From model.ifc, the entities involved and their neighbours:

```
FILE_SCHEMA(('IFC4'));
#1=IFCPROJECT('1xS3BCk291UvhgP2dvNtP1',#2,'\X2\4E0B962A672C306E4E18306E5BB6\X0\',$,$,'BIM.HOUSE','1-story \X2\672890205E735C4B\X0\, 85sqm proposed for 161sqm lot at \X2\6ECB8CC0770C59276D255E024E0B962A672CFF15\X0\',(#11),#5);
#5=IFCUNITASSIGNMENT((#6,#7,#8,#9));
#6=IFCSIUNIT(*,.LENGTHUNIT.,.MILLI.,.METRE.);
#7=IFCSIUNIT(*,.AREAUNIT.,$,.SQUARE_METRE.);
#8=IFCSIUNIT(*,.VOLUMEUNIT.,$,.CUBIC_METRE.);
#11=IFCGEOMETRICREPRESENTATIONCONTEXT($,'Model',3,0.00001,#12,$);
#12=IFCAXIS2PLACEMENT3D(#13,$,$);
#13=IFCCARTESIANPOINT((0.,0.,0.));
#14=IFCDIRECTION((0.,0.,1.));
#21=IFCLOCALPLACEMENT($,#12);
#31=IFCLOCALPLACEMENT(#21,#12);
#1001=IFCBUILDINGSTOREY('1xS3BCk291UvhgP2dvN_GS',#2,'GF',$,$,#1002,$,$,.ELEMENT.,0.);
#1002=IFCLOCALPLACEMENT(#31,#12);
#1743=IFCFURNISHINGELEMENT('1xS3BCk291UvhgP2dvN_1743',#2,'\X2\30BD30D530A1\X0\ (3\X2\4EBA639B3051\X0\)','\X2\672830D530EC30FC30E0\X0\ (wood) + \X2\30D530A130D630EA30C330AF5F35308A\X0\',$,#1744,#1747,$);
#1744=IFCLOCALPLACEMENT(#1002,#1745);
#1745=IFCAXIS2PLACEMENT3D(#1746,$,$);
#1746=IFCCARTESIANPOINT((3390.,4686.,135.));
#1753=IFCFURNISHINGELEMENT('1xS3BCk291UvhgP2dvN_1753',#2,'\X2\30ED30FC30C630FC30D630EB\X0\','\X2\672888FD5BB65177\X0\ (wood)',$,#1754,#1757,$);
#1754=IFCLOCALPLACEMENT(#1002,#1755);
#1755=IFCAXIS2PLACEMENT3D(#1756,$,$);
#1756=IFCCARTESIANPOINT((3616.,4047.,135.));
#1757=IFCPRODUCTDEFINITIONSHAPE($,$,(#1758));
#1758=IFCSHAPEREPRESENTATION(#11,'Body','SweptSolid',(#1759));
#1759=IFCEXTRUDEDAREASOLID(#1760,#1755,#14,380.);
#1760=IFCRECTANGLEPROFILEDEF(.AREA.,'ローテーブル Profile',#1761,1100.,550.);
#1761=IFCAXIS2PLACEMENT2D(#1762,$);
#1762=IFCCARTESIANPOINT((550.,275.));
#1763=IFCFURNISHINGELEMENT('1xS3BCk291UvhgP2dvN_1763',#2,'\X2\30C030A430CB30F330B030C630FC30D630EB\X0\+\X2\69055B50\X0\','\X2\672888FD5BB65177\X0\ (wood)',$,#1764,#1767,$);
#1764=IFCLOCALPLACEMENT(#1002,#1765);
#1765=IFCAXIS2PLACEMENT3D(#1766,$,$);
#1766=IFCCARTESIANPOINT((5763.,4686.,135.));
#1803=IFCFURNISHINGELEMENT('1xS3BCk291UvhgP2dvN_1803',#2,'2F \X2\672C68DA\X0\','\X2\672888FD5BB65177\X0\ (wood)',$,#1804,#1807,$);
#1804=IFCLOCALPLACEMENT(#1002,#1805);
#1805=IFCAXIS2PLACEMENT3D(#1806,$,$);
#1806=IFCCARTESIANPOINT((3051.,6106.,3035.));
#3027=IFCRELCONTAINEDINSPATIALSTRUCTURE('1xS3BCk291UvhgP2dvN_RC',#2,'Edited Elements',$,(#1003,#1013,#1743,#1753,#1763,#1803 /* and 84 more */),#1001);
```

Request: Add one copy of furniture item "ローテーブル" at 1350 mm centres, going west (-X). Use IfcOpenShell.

```python
import numpy as np
import ifcopenshell
import ifcopenshell.api.geometry
import ifcopenshell.api.root
import ifcopenshell.util.element
import ifcopenshell.util.placement
import ifcopenshell.util.unit

model = ifcopenshell.open("model.ifc")
unit_scale = ifcopenshell.util.unit.calculate_unit_scale(model)


def reuse_history(source, copy):
    """copy_class also copies each property set's owner history, people and application; keep the originals."""
    for rel in copy.IsDefinedBy:
        if rel.is_a("IfcRelDefinesByProperties") and (history := rel.RelatingPropertyDefinition.OwnerHistory):
            rel.RelatingPropertyDefinition.OwnerHistory = source.OwnerHistory
            ifcopenshell.util.element.remove_deep2(model, history)


source = model.by_guid("1xS3BCk291UvhgP2dvN_1753")
base = ifcopenshell.util.placement.get_local_placement(source.ObjectPlacement)
step = np.array([-1.0, 0.0, 0.0]) * 1.35 / unit_scale

for i in range(1, 2):
    copy = ifcopenshell.api.root.copy_class(model, product=source)
    copy.Representation = ifcopenshell.util.element.copy_deep(
        model, source.Representation, exclude=["IfcGeometricRepresentationContext", "IfcRepresentationMap"]
    )
    reuse_history(source, copy)
    matrix = base.copy()
    matrix[:3, 3] += i * step
    print("added at", matrix[:3, 3].round(3) + 0.0)
    ifcopenshell.api.geometry.edit_object_placement(model, product=copy, matrix=matrix, is_si=False)

model.write("model_v2.ifc")
```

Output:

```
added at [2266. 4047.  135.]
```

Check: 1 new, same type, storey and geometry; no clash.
